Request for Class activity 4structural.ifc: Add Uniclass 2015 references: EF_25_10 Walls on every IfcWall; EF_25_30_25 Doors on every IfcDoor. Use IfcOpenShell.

First a look at what the model holds.

```python
import ifcopenshell

model = ifcopenshell.open("Class activity 4structural.ifc")
print(model.schema)
print("classifications:", [c.Name for c in model.by_type("IfcClassification")])
for ifc_class in ("IfcDoor", "IfcRoof", "IfcStair", "IfcWall", "IfcWindow"):
    print(ifc_class, len(model.by_type(ifc_class)))
```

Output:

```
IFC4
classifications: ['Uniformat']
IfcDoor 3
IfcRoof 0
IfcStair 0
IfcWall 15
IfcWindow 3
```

```python
import ifcopenshell
import ifcopenshell.api.classification

model = ifcopenshell.open("Class activity 4structural.ifc")

system = ifcopenshell.api.classification.add_classification(model, classification="Uniclass 2015")

codes = {
    "IfcWall": ("EF_25_10", "Walls"),
    "IfcDoor": ("EF_25_30_25", "Doors"),
}
for ifc_class, (code, name) in codes.items():
    products = model.by_type(ifc_class)
    ifcopenshell.api.classification.add_reference(
        model, products=products, classification=system, identification=code, name=name
    )
    print(code, len(products))

model.write("Class activity 4structural_rev.ifc")
```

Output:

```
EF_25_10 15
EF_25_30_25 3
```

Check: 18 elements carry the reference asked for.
